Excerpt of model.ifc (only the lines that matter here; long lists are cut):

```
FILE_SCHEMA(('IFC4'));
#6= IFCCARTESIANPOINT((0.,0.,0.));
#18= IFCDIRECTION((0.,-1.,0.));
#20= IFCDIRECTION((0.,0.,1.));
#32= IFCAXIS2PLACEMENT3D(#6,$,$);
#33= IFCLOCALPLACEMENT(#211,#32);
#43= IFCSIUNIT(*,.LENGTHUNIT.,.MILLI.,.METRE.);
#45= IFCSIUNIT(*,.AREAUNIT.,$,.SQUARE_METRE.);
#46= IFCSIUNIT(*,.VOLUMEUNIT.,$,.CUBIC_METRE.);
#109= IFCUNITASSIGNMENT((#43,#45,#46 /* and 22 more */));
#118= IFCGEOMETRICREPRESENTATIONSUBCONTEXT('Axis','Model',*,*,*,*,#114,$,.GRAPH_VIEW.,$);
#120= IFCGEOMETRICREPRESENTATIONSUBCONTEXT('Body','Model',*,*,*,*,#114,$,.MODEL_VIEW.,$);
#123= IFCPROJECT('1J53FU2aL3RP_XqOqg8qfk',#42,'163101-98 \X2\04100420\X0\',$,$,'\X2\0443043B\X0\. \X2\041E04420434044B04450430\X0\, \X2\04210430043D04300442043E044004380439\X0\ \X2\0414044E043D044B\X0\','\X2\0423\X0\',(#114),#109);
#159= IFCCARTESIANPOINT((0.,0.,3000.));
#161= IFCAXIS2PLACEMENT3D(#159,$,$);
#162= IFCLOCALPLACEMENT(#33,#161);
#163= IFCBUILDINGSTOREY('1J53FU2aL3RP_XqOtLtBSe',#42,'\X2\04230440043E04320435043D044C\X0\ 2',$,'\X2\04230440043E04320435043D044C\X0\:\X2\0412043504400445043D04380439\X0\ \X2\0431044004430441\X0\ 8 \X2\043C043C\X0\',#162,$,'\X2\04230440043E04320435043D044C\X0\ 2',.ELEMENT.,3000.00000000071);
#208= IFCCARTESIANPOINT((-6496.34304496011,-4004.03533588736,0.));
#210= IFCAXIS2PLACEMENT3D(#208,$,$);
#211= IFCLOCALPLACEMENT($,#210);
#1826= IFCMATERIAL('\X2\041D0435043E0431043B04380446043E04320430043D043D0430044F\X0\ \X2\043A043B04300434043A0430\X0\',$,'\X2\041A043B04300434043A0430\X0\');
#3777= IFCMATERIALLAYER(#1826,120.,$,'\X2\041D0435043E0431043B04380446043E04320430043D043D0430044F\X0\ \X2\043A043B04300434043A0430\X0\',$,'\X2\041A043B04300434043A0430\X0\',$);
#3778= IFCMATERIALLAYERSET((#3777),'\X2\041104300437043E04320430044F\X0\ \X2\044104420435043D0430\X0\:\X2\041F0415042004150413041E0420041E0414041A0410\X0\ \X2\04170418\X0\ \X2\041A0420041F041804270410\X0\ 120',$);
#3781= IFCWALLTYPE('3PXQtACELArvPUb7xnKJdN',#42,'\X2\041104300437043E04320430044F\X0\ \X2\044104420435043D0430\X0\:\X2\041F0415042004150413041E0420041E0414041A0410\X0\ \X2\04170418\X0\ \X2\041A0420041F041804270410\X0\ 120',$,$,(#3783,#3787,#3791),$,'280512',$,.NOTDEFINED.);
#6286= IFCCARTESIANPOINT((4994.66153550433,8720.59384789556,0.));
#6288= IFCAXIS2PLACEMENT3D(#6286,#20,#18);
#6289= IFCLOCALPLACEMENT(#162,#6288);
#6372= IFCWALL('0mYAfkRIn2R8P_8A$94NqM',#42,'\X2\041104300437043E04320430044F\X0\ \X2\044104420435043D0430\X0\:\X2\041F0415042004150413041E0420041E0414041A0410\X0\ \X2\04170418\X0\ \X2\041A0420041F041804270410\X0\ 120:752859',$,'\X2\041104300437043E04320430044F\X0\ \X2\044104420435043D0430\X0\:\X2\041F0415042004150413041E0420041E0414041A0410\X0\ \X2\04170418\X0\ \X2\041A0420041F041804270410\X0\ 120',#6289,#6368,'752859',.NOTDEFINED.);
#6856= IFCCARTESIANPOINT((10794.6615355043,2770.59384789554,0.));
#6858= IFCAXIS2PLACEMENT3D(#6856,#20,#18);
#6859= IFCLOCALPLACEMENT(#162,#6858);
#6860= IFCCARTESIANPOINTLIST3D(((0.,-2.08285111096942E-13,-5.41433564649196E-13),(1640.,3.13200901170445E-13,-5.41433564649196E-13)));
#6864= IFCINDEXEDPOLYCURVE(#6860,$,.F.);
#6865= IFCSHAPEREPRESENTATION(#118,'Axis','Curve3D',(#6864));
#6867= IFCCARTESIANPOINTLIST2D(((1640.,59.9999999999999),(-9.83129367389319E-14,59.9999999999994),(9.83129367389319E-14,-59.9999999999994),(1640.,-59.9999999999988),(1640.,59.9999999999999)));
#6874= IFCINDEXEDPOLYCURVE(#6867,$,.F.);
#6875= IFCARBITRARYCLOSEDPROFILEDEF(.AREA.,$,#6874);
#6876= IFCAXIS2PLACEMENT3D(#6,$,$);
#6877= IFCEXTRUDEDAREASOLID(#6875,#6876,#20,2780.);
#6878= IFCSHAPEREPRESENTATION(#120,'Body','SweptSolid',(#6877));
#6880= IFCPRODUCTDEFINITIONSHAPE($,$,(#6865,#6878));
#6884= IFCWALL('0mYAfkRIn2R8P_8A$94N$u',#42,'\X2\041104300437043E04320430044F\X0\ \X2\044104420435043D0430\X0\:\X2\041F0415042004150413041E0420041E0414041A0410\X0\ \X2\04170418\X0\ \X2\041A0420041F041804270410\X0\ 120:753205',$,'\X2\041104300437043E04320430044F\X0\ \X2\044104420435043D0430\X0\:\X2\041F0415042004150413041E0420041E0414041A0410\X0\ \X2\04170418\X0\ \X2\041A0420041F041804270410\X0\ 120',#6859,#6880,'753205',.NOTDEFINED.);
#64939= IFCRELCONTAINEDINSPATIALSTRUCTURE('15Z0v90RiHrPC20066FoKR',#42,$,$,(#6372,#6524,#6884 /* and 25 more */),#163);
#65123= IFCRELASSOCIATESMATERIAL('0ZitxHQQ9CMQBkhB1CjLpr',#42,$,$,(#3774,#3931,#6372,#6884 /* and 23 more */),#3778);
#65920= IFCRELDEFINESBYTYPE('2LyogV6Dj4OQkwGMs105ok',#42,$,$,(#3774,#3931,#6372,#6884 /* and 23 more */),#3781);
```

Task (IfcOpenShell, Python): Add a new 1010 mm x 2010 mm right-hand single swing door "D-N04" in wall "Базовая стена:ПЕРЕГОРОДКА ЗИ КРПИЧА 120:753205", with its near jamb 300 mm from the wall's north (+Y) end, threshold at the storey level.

```python
import numpy as np
import ifcopenshell
import ifcopenshell.api.feature
import ifcopenshell.api.geometry
import ifcopenshell.api.root
import ifcopenshell.api.spatial
import ifcopenshell.geom
import ifcopenshell.util.element
import ifcopenshell.util.placement
import ifcopenshell.util.representation
import ifcopenshell.util.shape
import ifcopenshell.util.unit

model = ifcopenshell.open("model.ifc")
unit_scale = ifcopenshell.util.unit.calculate_unit_scale(model)
settings = ifcopenshell.geom.settings()


def volume(element):
    """Net volume in cubic metres, openings subtracted."""
    shape = ifcopenshell.geom.create_shape(settings, element)
    return ifcopenshell.util.shape.get_volume(shape.geometry)


wall = model.by_id(6884)
storey = ifcopenshell.util.element.get_container(wall, ifc_class="IfcBuildingStorey")
context = ifcopenshell.util.representation.get_context(model, "Model", "Body", "MODEL_VIEW")
before = volume(wall)

width, height, from_end, sill = 1.01, 2.01, 0.3, 0.0  # metres

# The wall runs along its own X axis, and the end named is its -X end.
wall_shape = ifcopenshell.geom.create_shape(settings, wall)
x, y, z = ifcopenshell.util.shape.get_vertices(wall_shape.geometry).T
start = x.min() + from_end
face, thickness = float(y.min()), float(y.max() - y.min())
wall_matrix = ifcopenshell.util.placement.get_local_placement(wall.ObjectPlacement)
level = ifcopenshell.util.placement.get_local_placement(storey.ObjectPlacement)[2, 3]


def in_wall(x, y):
    """Placement at x, y metres in the wall's axes, at sill height."""
    matrix = wall_matrix.copy()
    matrix[:, 3] = wall_matrix @ np.array([x / unit_scale, y / unit_scale, 0.0, 1.0])
    matrix[2, 3] = level + sill / unit_scale
    return matrix


# Opening: a box that overshoots both wall faces by 50 mm.
opening = ifcopenshell.api.root.create_entity(model, ifc_class="IfcOpeningElement", predefined_type="OPENING")
box = ifcopenshell.api.geometry.add_wall_representation(
    model, context=context, length=width, height=height, thickness=thickness + 0.1
)
ifcopenshell.api.geometry.assign_representation(model, product=opening, representation=box)
ifcopenshell.api.geometry.edit_object_placement(model, product=opening, matrix=in_wall(start, face - 0.05), is_si=False)
ifcopenshell.api.feature.add_feature(model, feature=opening, element=wall)

door = ifcopenshell.api.root.create_entity(model, ifc_class="IfcDoor", name="D-N04", predefined_type="DOOR")
door.OverallWidth, door.OverallHeight = width / unit_scale, height / unit_scale
door.OperationType = "SINGLE_SWING_RIGHT"
body = ifcopenshell.api.geometry.add_door_representation(
    model,
    context=context,
    overall_width=door.OverallWidth,
    overall_height=door.OverallHeight,
    operation_type="SINGLE_SWING_RIGHT",
    lining_properties={"LiningDepth": thickness / unit_scale, "ThresholdDepth": thickness / unit_scale},
)
ifcopenshell.api.geometry.assign_representation(model, product=door, representation=body)
ifcopenshell.api.spatial.assign_container(model, products=[door], relating_structure=storey)
ifcopenshell.api.feature.add_filling(model, opening=opening, element=door)

# The lining spans the wall, so the door starts at the wall face.
ifcopenshell.api.geometry.edit_object_placement(model, product=door, matrix=in_wall(start, face), is_si=False)

after = volume(wall)

print(f"wall volume {before:.3f} -> {after:.3f} m3")

model.write("model_v2.ifc")
```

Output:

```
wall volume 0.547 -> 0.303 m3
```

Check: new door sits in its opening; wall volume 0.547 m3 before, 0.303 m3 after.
